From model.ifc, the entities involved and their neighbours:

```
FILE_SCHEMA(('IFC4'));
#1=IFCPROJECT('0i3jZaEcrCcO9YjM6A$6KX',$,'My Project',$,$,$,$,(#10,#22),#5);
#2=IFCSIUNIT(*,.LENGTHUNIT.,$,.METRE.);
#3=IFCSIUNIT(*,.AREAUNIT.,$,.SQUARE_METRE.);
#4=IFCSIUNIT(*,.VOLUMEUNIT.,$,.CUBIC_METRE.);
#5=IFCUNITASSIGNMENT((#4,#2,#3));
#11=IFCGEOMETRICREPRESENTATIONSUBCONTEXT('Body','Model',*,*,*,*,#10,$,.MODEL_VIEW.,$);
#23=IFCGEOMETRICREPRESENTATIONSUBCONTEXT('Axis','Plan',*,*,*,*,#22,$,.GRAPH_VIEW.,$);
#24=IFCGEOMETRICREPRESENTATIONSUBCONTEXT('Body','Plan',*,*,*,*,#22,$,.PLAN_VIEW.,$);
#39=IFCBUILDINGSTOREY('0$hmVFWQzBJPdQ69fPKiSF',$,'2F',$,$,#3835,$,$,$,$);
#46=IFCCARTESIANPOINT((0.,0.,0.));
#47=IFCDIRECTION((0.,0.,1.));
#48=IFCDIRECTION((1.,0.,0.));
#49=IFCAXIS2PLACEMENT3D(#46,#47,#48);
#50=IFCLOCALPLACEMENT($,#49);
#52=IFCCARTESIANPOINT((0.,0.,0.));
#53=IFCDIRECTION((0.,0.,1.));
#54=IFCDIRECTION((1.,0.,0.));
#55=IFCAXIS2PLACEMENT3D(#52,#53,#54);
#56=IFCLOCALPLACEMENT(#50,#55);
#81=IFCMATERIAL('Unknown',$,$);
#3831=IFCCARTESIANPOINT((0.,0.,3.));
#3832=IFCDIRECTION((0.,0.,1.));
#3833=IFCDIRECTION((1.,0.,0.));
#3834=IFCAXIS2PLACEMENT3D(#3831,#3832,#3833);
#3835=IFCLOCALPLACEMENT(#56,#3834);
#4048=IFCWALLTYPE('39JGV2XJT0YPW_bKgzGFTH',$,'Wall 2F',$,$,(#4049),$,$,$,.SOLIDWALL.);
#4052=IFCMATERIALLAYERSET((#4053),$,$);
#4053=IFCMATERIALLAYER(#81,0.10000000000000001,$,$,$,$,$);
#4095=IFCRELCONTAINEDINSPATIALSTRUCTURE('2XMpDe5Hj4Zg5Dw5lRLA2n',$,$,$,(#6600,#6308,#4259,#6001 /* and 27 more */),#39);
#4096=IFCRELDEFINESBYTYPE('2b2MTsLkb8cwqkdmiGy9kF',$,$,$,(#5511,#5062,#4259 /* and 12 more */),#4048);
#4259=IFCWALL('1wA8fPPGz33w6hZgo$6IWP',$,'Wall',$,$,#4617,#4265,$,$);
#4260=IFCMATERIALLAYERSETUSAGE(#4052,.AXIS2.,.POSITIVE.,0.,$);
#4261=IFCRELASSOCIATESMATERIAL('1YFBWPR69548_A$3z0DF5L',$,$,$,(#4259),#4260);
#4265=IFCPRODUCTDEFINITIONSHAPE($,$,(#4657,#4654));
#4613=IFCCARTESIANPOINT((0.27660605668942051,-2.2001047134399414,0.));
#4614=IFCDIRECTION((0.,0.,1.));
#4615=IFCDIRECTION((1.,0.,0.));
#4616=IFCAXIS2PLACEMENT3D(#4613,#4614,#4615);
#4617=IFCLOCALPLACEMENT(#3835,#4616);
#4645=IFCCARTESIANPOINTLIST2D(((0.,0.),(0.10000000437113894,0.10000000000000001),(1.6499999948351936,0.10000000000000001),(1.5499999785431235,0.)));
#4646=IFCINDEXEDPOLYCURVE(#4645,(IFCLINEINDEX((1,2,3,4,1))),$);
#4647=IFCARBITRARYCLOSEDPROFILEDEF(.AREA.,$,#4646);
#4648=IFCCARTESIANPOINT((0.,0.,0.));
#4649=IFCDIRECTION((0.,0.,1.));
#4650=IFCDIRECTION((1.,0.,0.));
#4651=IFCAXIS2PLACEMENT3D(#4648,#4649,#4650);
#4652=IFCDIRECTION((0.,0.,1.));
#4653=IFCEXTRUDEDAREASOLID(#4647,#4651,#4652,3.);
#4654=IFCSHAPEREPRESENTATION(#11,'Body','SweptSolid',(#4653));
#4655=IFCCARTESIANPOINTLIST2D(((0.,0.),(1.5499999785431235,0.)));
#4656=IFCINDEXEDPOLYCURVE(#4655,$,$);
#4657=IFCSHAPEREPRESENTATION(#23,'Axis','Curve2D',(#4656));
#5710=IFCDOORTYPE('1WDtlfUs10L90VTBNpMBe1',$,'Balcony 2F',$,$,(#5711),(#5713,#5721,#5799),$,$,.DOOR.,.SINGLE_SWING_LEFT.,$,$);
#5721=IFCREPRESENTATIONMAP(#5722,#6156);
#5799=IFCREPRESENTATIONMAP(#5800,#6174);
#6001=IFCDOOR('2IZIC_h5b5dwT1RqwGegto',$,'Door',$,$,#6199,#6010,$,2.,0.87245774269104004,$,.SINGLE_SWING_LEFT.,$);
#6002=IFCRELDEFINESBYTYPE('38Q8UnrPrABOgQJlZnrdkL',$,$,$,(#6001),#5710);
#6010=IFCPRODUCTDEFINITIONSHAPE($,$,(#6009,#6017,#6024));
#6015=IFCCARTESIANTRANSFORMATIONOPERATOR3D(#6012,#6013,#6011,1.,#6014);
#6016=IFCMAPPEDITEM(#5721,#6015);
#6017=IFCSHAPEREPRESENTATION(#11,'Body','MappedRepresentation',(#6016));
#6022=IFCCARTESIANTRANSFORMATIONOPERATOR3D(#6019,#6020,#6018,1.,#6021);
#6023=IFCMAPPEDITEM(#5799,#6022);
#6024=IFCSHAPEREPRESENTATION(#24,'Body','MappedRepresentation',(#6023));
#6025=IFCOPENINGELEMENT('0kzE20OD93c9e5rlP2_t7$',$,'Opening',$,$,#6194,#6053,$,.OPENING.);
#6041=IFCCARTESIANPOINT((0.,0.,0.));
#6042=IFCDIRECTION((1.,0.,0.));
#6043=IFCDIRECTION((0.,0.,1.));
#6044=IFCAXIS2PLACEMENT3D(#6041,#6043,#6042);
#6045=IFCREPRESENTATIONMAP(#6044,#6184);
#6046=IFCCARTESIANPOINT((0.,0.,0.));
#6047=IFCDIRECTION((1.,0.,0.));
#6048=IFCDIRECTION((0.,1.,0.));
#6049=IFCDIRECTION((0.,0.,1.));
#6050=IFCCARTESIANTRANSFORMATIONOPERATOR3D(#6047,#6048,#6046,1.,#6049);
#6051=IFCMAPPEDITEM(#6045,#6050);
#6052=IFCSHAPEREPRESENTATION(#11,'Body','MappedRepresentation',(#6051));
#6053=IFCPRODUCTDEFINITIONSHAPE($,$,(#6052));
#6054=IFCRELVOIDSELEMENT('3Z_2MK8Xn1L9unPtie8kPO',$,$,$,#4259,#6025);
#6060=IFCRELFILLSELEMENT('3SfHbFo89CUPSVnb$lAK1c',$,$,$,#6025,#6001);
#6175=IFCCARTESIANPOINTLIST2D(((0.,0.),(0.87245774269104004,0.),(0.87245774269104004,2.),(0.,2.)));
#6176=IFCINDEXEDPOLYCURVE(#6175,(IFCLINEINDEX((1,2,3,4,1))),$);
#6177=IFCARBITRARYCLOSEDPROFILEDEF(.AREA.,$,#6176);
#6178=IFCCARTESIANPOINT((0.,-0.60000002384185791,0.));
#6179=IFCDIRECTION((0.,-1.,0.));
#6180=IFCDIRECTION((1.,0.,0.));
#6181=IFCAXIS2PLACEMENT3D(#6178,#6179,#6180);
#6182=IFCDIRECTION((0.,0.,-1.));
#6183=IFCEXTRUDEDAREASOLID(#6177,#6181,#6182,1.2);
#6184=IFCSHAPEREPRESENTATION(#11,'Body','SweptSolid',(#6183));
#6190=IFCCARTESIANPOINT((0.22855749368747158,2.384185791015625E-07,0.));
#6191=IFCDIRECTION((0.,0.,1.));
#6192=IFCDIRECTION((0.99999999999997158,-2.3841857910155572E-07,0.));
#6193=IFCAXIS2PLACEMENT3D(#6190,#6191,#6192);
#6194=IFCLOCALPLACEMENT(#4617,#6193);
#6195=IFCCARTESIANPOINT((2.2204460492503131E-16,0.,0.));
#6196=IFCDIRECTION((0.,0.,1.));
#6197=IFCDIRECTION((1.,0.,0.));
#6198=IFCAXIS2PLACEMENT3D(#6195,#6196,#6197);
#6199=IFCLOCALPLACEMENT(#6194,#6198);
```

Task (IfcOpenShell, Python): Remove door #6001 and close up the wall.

```python
import ifcopenshell
import ifcopenshell.api.feature
import ifcopenshell.api.root
import ifcopenshell.geom
import ifcopenshell.util.shape

model = ifcopenshell.open("model.ifc")
settings = ifcopenshell.geom.settings()


def volume(element):
    """Net volume in cubic metres, openings subtracted."""
    shape = ifcopenshell.geom.create_shape(settings, element)
    return ifcopenshell.util.shape.get_volume(shape.geometry)


door = model.by_guid("2IZIC_h5b5dwT1RqwGegto")
opening = door.FillsVoids[0].RelatingOpeningElement
wall = opening.VoidsElements[0].RelatingBuildingElement
before = volume(wall)

ifcopenshell.api.root.remove_product(model, product=door)
ifcopenshell.api.feature.remove_feature(model, feature=opening)

after = volume(wall)

print(f"wall volume {before:.3f} -> {after:.3f} m3")

model.write("model_rev.ifc")
```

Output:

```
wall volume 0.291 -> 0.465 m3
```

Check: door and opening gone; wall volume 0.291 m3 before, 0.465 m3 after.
